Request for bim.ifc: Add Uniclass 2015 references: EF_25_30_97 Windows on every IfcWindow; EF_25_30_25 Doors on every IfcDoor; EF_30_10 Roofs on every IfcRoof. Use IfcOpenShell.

First a look at what the model holds.

```python
import ifcopenshell

model = ifcopenshell.open("bim.ifc")
print(model.schema)
print("classifications:", [c.Name for c in model.by_type("IfcClassification")])
for ifc_class in ("IfcDoor", "IfcRoof", "IfcStair", "IfcWall", "IfcWindow"):
    print(ifc_class, len(model.by_type(ifc_class)))
```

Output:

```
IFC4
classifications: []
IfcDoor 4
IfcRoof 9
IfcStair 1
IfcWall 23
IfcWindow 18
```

```python
import ifcopenshell
import ifcopenshell.api.classification

model = ifcopenshell.open("bim.ifc")

system = ifcopenshell.api.classification.add_classification(model, classification="Uniclass 2015")

codes = {
    "IfcWindow": ("EF_25_30_97", "Windows"),
    "IfcDoor": ("EF_25_30_25", "Doors"),
    "IfcRoof": ("EF_30_10", "Roofs"),
}
for ifc_class, (code, name) in codes.items():
    products = model.by_type(ifc_class)
    ifcopenshell.api.classification.add_reference(
        model, products=products, classification=system, identification=code, name=name
    )
    print(code, len(products))

model.write("bim_rev.ifc")
```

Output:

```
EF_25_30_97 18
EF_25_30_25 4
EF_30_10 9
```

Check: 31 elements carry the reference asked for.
